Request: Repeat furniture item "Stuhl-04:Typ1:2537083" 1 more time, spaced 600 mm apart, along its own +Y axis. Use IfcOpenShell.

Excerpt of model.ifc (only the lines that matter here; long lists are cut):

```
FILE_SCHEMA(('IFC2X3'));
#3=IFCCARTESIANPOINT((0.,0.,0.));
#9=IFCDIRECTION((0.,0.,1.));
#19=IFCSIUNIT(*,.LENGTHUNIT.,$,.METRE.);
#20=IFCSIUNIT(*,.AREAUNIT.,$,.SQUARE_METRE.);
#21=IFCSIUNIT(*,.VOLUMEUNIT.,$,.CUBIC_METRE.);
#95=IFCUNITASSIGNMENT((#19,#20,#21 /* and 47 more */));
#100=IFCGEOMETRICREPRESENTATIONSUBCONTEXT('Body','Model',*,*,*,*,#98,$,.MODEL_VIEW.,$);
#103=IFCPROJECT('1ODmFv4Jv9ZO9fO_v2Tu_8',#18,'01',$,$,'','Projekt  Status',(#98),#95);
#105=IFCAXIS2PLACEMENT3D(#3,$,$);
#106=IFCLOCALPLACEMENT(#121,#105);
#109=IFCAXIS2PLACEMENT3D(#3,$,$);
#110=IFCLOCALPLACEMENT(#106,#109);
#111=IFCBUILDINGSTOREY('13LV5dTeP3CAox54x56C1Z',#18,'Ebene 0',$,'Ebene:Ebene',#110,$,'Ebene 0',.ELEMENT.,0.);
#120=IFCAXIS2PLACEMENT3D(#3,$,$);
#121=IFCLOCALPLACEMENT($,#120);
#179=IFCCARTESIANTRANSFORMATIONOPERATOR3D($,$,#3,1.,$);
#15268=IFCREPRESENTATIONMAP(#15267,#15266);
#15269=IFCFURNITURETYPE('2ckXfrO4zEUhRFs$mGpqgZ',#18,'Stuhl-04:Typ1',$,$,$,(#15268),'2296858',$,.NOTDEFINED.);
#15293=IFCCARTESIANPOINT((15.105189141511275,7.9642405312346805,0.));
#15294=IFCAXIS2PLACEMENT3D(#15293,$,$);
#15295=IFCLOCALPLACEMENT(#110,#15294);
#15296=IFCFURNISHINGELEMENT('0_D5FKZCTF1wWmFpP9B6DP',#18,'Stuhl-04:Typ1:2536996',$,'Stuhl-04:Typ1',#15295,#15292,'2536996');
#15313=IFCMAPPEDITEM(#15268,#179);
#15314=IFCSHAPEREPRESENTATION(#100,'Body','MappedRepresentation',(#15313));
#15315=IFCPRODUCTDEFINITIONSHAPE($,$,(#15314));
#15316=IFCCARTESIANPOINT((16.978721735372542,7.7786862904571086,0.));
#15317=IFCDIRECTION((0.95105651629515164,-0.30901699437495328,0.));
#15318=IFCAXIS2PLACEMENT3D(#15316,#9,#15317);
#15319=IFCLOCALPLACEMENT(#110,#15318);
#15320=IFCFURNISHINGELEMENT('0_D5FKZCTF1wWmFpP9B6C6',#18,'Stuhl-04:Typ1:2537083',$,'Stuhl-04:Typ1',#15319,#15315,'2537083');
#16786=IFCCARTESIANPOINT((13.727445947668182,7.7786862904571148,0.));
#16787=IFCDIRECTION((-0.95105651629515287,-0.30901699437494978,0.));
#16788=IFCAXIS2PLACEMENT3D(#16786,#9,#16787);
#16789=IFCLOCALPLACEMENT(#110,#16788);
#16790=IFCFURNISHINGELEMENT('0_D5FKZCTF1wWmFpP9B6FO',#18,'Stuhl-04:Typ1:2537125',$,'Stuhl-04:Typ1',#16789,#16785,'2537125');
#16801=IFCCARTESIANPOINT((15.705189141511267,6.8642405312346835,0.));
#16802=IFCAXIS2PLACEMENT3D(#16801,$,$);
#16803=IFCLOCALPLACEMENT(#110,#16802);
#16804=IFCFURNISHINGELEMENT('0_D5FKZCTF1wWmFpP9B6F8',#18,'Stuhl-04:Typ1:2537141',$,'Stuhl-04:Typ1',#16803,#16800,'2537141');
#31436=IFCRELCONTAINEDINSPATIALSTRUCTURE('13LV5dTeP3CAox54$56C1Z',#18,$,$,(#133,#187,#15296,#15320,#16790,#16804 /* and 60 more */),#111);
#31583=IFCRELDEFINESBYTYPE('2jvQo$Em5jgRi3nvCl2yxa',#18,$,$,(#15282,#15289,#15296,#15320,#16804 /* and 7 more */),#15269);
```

```python
import ifcopenshell
import ifcopenshell.api.geometry
import ifcopenshell.api.root
import ifcopenshell.util.element
import ifcopenshell.util.placement

model = ifcopenshell.open("model.ifc")

source = model.by_id(15320)
base = ifcopenshell.util.placement.get_local_placement(source.ObjectPlacement)
step = base[:3, 1] * 0.6

for i in range(1, 2):
    copy = ifcopenshell.api.root.copy_class(model, product=source)
    copy.Representation = ifcopenshell.util.element.copy_deep(
        model, source.Representation, exclude=["IfcGeometricRepresentationContext", "IfcRepresentationMap"]
    )
    copy.Name = "Stuhl-04:Typ1"
    copy.Tag = None
    matrix = base.copy()
    matrix[:3, 3] += i * step
    print("added at", matrix[:3, 3].round(3) + 0.0)
    ifcopenshell.api.geometry.edit_object_placement(model, product=copy, matrix=matrix, is_si=False)

model.write("model_edited.ifc")
```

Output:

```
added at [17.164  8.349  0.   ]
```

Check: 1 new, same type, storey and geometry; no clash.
